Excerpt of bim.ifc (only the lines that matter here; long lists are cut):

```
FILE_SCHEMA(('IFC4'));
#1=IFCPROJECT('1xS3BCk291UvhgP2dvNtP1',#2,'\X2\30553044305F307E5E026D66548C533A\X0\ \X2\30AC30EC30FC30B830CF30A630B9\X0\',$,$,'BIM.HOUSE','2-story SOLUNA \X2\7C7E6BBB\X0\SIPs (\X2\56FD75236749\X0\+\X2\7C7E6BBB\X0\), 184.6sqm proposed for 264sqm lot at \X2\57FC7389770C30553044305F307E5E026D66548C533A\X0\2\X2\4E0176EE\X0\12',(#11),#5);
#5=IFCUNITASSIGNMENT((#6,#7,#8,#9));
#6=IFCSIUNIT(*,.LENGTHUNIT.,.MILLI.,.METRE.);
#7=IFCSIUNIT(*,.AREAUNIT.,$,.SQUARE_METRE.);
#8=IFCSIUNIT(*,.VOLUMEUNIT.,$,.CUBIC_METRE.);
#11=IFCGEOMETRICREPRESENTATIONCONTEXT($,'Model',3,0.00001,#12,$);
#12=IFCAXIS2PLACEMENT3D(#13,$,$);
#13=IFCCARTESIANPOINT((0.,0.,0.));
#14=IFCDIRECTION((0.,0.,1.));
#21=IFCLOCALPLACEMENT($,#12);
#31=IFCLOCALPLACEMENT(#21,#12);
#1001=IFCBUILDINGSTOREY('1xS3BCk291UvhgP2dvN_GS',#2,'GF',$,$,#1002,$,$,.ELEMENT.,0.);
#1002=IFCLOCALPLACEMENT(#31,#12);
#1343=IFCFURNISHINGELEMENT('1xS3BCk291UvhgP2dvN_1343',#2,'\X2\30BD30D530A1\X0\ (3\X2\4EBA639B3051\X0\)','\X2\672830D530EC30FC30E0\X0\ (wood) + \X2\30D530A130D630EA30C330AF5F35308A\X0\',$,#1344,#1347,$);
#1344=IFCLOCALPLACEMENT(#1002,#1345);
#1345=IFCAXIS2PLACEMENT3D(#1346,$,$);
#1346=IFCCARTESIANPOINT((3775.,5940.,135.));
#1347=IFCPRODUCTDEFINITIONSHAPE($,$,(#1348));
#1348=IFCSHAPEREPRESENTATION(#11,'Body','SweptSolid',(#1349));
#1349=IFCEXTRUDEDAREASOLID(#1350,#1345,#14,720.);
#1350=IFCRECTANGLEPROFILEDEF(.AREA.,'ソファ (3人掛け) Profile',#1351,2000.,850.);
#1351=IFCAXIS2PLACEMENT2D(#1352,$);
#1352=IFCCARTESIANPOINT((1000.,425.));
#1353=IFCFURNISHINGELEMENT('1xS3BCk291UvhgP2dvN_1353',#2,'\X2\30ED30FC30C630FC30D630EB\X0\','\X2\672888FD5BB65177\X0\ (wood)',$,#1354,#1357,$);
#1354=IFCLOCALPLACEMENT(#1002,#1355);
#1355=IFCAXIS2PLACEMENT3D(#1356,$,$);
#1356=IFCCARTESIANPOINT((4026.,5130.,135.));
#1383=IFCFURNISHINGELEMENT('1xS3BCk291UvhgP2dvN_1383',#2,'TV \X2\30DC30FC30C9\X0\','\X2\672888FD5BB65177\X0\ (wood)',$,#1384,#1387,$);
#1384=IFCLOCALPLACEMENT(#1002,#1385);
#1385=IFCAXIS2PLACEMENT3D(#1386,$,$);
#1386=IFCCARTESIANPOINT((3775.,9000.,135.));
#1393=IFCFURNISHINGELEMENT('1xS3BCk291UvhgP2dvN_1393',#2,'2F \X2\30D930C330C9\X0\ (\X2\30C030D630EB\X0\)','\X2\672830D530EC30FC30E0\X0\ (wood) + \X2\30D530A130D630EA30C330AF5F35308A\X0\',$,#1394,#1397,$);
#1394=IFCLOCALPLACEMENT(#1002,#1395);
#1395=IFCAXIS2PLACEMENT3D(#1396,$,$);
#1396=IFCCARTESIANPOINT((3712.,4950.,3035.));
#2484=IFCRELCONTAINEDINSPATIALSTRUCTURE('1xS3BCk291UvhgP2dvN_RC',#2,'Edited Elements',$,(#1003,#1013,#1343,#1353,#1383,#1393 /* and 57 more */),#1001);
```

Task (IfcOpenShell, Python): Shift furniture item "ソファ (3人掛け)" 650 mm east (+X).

```python
import ifcopenshell
import ifcopenshell.api.geometry
import ifcopenshell.util.placement
import ifcopenshell.util.unit

model = ifcopenshell.open("bim.ifc")
unit_scale = ifcopenshell.util.unit.calculate_unit_scale(model)

item = model.by_guid("1xS3BCk291UvhgP2dvN_1343")
matrix = ifcopenshell.util.placement.get_local_placement(item.ObjectPlacement)
matrix[0, 3] += 0.65 / unit_scale
ifcopenshell.api.geometry.edit_object_placement(model, product=item, matrix=matrix, is_si=False)

print(ifcopenshell.util.placement.get_local_placement(item.ObjectPlacement).round(3) + 0.0)

model.write("bim_v2.ifc")
```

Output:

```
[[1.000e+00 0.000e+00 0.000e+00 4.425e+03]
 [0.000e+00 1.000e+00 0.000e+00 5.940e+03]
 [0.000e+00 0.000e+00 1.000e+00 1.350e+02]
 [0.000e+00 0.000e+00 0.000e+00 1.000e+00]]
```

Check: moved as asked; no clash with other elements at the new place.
